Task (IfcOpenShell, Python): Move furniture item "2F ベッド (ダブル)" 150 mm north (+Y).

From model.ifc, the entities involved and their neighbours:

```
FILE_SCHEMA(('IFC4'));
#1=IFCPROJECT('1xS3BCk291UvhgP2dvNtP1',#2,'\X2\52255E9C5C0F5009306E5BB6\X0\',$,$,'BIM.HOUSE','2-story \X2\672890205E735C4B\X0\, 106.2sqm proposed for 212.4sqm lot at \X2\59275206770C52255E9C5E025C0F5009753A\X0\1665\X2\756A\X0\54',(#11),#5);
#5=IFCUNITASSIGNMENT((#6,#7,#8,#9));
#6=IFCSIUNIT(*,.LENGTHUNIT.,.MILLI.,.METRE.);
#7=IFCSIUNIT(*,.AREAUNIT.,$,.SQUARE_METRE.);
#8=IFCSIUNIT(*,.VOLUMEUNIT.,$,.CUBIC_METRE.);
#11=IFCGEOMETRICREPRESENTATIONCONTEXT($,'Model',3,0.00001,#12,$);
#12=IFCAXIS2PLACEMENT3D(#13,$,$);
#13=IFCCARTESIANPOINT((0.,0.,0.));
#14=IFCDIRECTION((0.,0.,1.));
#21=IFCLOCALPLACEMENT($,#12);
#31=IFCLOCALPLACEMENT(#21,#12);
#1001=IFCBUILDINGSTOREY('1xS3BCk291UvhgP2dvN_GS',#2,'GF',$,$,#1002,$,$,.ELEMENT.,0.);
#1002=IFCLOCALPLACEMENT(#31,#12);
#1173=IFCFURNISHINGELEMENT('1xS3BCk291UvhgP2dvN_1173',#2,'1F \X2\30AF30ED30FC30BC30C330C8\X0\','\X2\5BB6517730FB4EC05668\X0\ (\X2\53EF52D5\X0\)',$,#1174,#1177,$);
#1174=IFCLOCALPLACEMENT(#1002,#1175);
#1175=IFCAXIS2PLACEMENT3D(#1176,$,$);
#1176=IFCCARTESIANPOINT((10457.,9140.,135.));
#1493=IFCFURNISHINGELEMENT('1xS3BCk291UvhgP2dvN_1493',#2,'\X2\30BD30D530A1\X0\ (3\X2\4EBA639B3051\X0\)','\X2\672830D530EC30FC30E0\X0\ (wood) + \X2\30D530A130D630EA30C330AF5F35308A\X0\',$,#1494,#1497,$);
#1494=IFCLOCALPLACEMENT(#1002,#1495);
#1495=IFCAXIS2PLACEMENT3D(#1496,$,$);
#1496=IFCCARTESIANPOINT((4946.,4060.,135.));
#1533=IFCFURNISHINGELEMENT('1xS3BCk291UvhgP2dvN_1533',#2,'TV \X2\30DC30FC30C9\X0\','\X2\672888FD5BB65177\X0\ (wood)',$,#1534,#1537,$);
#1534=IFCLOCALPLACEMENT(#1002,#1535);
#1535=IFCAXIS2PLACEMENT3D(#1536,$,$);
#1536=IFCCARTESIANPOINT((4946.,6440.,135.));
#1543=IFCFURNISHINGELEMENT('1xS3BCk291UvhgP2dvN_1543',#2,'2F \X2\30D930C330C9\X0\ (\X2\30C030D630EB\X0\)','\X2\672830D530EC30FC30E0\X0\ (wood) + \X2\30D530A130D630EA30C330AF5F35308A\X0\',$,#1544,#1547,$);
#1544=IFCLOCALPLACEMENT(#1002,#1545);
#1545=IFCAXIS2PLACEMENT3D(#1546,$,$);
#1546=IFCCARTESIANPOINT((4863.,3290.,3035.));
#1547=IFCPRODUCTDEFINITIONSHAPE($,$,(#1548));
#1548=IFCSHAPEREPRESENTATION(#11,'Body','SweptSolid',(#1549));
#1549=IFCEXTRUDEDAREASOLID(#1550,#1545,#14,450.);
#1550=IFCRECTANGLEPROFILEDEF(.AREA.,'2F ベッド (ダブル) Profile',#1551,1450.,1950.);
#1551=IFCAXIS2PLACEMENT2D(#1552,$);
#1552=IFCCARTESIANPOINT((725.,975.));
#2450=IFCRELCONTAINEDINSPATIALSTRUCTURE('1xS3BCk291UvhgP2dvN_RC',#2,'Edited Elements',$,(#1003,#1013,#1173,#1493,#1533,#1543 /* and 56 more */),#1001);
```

```python
import ifcopenshell
import ifcopenshell.api.geometry
import ifcopenshell.util.placement

model = ifcopenshell.open("model.ifc")

item = model.by_guid("1xS3BCk291UvhgP2dvN_1543")
matrix = ifcopenshell.util.placement.get_local_placement(item.ObjectPlacement)
matrix[1, 3] += 150.0
ifcopenshell.api.geometry.edit_object_placement(model, product=item, matrix=matrix, is_si=False)

print(ifcopenshell.util.placement.get_local_placement(item.ObjectPlacement).round(3) + 0.0)

model.write("model_updated.ifc")
```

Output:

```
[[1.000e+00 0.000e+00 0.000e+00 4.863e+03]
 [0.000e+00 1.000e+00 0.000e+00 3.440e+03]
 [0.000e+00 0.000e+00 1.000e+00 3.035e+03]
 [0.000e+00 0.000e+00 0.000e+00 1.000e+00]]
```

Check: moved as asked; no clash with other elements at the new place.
